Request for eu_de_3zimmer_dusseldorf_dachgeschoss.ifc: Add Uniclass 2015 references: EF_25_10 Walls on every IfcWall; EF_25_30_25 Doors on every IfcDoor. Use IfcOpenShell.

First a look at what the model holds.

```python
import ifcopenshell

model = ifcopenshell.open("eu_de_3zimmer_dusseldorf_dachgeschoss.ifc")
print(model.schema)
print("classifications:", [c.Name for c in model.by_type("IfcClassification")])
for ifc_class in ("IfcDoor", "IfcRoof", "IfcStair", "IfcWall", "IfcWindow"):
    print(ifc_class, len(model.by_type(ifc_class)))
```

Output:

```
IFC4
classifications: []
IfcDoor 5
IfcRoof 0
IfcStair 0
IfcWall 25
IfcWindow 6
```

```python
import ifcopenshell
import ifcopenshell.api.classification

model = ifcopenshell.open("eu_de_3zimmer_dusseldorf_dachgeschoss.ifc")

system = ifcopenshell.api.classification.add_classification(model, classification="Uniclass 2015")

codes = {
    "IfcWall": ("EF_25_10", "Walls"),
    "IfcDoor": ("EF_25_30_25", "Doors"),
}
for ifc_class, (code, name) in codes.items():
    products = model.by_type(ifc_class)
    ifcopenshell.api.classification.add_reference(
        model, products=products, classification=system, identification=code, name=name
    )
    print(code, len(products))

model.write("eu_de_3zimmer_dusseldorf_dachgeschoss-out.ifc")
```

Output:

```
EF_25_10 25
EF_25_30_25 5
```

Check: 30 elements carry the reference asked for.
